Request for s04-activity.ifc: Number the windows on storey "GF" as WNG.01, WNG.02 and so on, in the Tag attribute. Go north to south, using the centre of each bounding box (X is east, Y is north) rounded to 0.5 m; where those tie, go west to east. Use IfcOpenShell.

First a look at what the model holds.

```python
import ifcopenshell
import ifcopenshell.util.element
import ifcopenshell.util.placement

model = ifcopenshell.open("s04-activity.ifc")
print(model.schema)
storey = next(s for s in model.by_type("IfcBuildingStorey") if s.Name == "GF")
windows = [e for e in ifcopenshell.util.element.get_decomposition(storey) if e.is_a("IfcWindow")]
for e in sorted(windows, key=lambda e: e.id()):
    origin = ifcopenshell.util.placement.get_local_placement(e.ObjectPlacement)[:3, 3]
    print(e.id(), e.Tag, e.Name, origin.round(2) + 0.0, sep=" | ")
```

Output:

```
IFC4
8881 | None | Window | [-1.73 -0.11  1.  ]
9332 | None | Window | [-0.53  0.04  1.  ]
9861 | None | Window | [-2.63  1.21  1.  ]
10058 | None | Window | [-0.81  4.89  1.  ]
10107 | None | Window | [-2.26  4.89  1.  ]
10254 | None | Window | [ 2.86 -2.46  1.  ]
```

```python
import ifcopenshell
import ifcopenshell.geom
import ifcopenshell.util.element
import ifcopenshell.util.shape

model = ifcopenshell.open("s04-activity.ifc")
settings = ifcopenshell.geom.settings()
settings.set("use-world-coords", True)


def centre(element):
    shape = ifcopenshell.geom.create_shape(settings, element)
    return ifcopenshell.util.shape.get_bbox_centroid(shape.geometry)


storey = next(s for s in model.by_type("IfcBuildingStorey") if s.Name == "GF")
windows = [e for e in ifcopenshell.util.element.get_decomposition(storey) if e.is_a("IfcWindow")]

# Insertion points can sit at a corner or the storey origin, so sort by the geometry (in metres).
centres = {e: centre(e) for e in windows}
windows.sort(key=lambda e: (-round(centres[e][1] / 0.5), centres[e][0]))

for i, e in enumerate(windows, start=1):
    number = f"WNG.{i:02d}"
    e.Tag = number
    print(e.id(), number)

model.write("s04-activity-out.ifc")
```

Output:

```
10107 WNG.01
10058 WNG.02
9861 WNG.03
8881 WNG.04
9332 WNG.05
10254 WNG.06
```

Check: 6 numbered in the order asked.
